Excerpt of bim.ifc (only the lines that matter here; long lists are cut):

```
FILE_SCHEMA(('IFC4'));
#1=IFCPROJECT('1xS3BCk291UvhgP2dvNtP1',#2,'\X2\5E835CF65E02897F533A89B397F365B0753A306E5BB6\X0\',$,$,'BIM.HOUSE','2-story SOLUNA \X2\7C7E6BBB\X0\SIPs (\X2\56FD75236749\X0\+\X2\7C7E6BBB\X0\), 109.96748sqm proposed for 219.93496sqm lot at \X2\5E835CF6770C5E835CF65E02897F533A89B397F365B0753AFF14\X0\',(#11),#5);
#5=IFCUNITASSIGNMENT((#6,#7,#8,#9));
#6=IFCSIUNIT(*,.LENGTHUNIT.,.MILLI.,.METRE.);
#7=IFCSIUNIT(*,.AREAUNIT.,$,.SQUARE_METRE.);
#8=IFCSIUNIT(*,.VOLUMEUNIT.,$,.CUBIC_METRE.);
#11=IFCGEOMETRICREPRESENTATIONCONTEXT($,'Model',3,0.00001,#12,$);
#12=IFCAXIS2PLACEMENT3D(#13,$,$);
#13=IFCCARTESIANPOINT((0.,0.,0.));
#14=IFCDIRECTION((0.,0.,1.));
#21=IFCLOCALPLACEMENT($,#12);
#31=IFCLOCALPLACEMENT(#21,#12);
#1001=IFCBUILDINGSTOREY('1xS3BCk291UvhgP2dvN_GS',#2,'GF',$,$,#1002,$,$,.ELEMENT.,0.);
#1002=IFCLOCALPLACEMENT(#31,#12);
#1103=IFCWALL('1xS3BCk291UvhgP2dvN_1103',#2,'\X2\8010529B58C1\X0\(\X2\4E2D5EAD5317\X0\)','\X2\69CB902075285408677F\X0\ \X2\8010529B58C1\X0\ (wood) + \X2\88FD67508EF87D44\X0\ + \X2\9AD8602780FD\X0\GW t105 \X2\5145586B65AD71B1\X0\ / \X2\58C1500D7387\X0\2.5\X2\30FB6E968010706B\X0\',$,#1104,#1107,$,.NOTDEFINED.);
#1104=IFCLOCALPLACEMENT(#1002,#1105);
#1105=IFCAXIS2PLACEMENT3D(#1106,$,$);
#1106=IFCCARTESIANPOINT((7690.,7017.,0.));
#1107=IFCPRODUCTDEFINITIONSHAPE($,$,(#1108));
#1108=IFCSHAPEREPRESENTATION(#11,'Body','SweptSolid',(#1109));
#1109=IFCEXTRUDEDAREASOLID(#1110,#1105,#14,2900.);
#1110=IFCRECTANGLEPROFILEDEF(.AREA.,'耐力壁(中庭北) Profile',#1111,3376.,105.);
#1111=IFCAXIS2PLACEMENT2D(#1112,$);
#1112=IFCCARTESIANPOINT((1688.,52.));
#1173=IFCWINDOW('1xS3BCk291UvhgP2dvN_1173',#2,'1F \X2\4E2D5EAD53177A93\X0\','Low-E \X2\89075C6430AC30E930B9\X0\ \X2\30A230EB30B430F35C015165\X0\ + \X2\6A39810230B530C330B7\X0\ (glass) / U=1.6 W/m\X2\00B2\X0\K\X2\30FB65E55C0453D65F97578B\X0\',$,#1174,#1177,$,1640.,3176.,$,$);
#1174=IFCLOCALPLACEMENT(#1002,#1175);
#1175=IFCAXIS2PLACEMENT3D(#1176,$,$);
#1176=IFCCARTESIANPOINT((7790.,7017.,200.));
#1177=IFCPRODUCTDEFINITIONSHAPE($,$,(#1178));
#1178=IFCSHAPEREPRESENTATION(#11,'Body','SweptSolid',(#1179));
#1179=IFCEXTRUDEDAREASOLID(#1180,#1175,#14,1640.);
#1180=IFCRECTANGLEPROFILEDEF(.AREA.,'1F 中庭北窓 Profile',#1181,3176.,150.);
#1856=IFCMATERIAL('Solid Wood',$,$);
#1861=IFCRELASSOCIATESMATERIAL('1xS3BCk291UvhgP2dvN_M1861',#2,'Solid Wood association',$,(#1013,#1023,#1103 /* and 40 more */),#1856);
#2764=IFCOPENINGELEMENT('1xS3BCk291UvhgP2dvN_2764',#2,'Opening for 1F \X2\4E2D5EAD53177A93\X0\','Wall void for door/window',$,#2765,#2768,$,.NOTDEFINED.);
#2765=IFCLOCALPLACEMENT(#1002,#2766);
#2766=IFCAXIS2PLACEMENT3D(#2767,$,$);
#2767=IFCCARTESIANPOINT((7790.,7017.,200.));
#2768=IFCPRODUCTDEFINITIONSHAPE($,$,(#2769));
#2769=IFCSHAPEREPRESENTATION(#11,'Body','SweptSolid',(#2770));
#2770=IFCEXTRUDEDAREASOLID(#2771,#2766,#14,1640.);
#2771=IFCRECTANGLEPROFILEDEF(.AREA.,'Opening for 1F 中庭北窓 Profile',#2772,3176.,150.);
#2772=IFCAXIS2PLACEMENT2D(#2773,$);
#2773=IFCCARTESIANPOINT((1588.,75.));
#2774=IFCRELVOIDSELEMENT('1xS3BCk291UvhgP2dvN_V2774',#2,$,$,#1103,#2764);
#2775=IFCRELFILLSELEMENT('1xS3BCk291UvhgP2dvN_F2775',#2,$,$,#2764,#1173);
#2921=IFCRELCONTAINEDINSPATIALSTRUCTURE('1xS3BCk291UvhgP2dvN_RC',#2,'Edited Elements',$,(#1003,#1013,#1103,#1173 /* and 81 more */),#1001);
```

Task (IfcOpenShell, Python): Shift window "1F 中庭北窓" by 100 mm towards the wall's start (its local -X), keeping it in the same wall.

```python
import ifcopenshell
import ifcopenshell.api.geometry
import ifcopenshell.util.placement

model = ifcopenshell.open("bim.ifc")

window = model.by_guid("1xS3BCk291UvhgP2dvN_1173")
opening = window.FillsVoids[0].RelatingOpeningElement
wall = opening.VoidsElements[0].RelatingBuildingElement

wall_matrix = ifcopenshell.util.placement.get_local_placement(wall.ObjectPlacement)
shift = wall_matrix[:3, 0] * -100.0
before = ifcopenshell.util.placement.get_local_placement(window.ObjectPlacement)[:3, 3].copy()

# The window is not placed relative to its opening, so move both.
for product in (opening, window):
    matrix = ifcopenshell.util.placement.get_local_placement(product.ObjectPlacement)
    matrix[:3, 3] += shift
    ifcopenshell.api.geometry.edit_object_placement(model, product=product, matrix=matrix, is_si=False)

after = ifcopenshell.util.placement.get_local_placement(window.ObjectPlacement)[:3, 3]
print("window moved by", (after - before).round(3) + 0.0)

model.write("bim_rev.ifc")
```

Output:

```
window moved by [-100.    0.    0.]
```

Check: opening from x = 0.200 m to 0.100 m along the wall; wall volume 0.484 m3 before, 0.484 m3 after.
